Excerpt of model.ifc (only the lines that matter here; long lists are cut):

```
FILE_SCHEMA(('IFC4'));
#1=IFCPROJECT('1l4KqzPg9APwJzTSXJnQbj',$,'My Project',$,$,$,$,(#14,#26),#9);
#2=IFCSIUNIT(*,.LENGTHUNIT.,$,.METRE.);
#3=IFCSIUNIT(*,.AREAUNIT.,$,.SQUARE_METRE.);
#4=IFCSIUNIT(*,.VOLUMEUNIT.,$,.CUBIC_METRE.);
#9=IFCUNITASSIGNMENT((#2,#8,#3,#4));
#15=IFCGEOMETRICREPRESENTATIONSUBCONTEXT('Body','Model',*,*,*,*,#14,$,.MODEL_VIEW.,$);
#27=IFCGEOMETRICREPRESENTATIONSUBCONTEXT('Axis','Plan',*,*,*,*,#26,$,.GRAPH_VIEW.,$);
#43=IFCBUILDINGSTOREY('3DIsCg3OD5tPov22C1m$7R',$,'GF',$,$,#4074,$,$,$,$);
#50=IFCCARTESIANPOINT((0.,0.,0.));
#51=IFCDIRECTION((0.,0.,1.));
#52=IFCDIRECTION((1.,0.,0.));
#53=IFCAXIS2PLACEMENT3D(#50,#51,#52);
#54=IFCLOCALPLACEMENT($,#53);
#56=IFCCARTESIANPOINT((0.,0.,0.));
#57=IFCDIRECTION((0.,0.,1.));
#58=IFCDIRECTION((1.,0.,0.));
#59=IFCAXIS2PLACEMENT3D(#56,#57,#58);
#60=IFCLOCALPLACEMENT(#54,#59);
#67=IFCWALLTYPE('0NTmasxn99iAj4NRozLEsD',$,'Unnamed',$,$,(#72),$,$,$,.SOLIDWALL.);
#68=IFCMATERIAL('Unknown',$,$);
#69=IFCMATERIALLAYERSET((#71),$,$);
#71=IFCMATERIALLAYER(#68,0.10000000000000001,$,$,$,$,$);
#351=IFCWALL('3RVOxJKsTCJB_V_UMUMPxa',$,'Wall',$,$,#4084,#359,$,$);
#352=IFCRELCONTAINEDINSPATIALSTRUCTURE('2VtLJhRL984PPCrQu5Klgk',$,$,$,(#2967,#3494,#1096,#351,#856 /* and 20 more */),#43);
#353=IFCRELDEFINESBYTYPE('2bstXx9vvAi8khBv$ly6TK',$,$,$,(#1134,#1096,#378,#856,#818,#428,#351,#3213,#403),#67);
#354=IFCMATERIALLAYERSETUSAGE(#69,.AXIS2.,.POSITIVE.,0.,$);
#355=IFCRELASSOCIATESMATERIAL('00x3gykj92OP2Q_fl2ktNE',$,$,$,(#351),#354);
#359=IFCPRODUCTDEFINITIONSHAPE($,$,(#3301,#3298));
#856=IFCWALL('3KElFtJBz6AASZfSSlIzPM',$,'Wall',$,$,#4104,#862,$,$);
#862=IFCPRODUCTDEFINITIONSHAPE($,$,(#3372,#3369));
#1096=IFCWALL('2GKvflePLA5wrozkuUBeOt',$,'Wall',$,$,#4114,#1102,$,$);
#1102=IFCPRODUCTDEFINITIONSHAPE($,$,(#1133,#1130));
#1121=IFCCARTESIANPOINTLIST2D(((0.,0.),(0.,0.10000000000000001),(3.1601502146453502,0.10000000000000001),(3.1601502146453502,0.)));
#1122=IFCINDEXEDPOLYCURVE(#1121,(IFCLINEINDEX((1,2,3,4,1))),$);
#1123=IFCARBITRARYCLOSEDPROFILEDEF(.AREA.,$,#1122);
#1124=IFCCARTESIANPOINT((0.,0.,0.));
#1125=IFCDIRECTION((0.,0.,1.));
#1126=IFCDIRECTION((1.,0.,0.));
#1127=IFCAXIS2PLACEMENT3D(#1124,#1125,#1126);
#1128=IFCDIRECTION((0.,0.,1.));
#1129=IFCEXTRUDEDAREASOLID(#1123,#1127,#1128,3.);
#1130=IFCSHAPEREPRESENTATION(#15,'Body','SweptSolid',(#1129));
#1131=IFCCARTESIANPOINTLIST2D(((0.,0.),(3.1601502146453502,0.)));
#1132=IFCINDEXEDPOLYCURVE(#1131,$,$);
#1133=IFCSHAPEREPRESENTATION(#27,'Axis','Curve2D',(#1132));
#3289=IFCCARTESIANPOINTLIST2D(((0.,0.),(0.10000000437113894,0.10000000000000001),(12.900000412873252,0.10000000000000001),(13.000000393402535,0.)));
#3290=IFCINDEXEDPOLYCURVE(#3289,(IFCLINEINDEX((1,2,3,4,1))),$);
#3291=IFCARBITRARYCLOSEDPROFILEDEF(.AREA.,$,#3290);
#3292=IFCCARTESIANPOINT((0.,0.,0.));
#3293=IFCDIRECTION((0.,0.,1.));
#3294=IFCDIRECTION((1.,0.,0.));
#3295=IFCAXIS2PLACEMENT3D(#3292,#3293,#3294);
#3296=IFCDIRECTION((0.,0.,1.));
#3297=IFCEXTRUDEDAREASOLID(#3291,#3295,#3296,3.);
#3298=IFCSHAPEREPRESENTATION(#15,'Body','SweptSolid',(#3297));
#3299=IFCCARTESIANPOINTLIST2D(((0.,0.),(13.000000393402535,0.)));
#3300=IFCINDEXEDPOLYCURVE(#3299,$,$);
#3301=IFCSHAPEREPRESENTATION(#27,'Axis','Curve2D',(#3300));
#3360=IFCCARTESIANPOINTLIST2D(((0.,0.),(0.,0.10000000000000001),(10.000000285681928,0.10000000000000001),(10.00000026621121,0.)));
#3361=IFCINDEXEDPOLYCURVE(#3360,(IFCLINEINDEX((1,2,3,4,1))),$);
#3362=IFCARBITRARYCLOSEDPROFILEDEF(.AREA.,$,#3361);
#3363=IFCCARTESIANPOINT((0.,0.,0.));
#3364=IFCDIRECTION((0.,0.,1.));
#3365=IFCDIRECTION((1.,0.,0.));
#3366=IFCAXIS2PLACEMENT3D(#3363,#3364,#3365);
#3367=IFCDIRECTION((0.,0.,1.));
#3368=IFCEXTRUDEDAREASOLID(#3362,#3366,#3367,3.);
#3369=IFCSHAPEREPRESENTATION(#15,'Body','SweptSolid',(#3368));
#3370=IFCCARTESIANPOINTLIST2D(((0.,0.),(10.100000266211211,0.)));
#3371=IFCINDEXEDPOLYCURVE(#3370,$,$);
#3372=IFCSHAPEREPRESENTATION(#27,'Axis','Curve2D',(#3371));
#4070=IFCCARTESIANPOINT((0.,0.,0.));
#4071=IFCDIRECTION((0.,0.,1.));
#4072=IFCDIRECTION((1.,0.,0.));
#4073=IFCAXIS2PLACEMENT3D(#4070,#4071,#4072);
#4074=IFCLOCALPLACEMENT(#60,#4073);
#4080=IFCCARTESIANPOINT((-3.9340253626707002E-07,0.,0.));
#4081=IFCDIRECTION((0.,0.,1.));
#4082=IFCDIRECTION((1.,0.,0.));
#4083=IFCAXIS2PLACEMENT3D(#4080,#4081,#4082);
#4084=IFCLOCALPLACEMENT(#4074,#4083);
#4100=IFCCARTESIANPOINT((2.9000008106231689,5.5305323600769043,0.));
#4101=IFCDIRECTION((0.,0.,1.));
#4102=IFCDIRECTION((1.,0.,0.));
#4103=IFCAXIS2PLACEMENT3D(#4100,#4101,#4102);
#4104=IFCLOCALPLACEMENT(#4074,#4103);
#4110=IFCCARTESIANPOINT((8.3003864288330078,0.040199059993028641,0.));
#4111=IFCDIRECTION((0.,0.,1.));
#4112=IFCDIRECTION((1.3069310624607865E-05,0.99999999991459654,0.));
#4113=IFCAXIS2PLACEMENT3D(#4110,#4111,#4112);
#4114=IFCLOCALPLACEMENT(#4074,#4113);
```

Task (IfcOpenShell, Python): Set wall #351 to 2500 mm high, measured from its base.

```python
import ifcopenshell
import ifcopenshell.geom
import ifcopenshell.util.representation
import ifcopenshell.util.shape

model = ifcopenshell.open("model.ifc")
settings = ifcopenshell.geom.settings()


def volume(element):
    """Net volume in cubic metres, openings subtracted."""
    shape = ifcopenshell.geom.create_shape(settings, element)
    return ifcopenshell.util.shape.get_volume(shape.geometry)


wall = model.by_guid("3RVOxJKsTCJB_V_UMUMPxa")
before = volume(wall)

body = ifcopenshell.util.representation.get_representation(wall, "Model", "Body")
solid = body.Items[0]
old_height = solid.Depth
solid.Depth = 2.5
after = volume(wall)

print(f"height {old_height:g} -> {solid.Depth:g}, volume {before:.3f} -> {after:.3f} m3")

model.write("model_rev.ifc")
```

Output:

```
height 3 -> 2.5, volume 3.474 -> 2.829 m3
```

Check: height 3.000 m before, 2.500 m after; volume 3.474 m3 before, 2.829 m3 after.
